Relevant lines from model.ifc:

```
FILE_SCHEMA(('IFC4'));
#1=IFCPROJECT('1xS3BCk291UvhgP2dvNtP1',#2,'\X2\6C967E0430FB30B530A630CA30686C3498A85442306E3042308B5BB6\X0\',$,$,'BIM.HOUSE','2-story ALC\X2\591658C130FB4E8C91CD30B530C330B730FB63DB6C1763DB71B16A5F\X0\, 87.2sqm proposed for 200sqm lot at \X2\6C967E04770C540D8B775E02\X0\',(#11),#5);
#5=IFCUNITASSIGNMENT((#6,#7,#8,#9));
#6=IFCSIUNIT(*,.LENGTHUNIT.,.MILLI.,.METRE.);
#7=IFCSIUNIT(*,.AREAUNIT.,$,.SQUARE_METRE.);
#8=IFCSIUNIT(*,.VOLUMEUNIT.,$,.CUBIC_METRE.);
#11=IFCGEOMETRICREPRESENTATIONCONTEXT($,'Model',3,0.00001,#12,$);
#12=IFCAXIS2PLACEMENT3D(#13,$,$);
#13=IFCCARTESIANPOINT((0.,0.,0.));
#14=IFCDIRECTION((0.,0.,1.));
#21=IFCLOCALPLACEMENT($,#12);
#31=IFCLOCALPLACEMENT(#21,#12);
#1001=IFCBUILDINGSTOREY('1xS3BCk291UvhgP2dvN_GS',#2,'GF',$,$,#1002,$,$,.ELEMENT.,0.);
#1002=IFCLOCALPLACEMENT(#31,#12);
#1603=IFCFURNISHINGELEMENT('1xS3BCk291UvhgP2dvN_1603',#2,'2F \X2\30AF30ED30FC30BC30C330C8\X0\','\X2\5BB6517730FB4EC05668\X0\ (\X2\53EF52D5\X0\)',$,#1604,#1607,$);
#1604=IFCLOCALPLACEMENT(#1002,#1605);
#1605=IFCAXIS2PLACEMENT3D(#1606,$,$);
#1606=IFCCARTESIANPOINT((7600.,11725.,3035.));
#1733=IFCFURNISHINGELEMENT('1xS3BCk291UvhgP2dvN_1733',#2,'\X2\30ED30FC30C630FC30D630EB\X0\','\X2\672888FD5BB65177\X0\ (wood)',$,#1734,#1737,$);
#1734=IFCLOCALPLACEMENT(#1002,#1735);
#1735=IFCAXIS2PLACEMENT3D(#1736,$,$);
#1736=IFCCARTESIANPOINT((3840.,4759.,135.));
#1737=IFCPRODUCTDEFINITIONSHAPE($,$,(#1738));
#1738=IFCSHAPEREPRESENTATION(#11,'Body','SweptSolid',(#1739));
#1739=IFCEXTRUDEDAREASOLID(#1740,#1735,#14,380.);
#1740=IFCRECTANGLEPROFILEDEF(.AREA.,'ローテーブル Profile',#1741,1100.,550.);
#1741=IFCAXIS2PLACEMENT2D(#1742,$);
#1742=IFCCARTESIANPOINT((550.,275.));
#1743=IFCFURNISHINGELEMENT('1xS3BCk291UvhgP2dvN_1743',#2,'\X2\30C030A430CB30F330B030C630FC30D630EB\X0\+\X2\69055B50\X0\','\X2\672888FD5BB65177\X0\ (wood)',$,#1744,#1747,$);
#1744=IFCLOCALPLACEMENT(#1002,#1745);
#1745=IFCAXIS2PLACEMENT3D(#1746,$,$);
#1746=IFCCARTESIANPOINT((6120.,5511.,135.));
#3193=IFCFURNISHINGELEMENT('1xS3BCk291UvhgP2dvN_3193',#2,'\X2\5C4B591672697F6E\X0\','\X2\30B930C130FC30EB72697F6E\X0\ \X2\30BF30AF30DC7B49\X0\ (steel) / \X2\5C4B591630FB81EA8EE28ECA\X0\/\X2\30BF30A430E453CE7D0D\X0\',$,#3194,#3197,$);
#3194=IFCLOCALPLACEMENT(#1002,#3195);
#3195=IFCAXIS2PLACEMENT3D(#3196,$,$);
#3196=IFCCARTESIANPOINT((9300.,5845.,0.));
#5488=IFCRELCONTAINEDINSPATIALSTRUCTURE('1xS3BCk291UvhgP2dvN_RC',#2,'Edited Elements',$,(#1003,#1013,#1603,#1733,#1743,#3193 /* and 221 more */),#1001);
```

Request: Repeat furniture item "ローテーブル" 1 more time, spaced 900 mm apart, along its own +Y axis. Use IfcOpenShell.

```python
import ifcopenshell
import ifcopenshell.api.geometry
import ifcopenshell.api.root
import ifcopenshell.util.element
import ifcopenshell.util.placement

model = ifcopenshell.open("model.ifc")


def reuse_history(source, copy):
    """copy_class also copies each property set's owner history, people and application; keep the originals."""
    for rel in copy.IsDefinedBy:
        if rel.is_a("IfcRelDefinesByProperties") and (history := rel.RelatingPropertyDefinition.OwnerHistory):
            rel.RelatingPropertyDefinition.OwnerHistory = source.OwnerHistory
            ifcopenshell.util.element.remove_deep2(model, history)


source = model.by_guid("1xS3BCk291UvhgP2dvN_1733")
base = ifcopenshell.util.placement.get_local_placement(source.ObjectPlacement)
step = base[:3, 1] * 900.0

for i in range(1, 2):
    copy = ifcopenshell.api.root.copy_class(model, product=source)
    copy.Representation = ifcopenshell.util.element.copy_deep(
        model, source.Representation, exclude=["IfcGeometricRepresentationContext", "IfcRepresentationMap"]
    )
    reuse_history(source, copy)
    matrix = base.copy()
    matrix[:3, 3] += i * step
    print("added at", matrix[:3, 3].round(3) + 0.0)
    ifcopenshell.api.geometry.edit_object_placement(model, product=copy, matrix=matrix, is_si=False)

model.write("model-out.ifc")
```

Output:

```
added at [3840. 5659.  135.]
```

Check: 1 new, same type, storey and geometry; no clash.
